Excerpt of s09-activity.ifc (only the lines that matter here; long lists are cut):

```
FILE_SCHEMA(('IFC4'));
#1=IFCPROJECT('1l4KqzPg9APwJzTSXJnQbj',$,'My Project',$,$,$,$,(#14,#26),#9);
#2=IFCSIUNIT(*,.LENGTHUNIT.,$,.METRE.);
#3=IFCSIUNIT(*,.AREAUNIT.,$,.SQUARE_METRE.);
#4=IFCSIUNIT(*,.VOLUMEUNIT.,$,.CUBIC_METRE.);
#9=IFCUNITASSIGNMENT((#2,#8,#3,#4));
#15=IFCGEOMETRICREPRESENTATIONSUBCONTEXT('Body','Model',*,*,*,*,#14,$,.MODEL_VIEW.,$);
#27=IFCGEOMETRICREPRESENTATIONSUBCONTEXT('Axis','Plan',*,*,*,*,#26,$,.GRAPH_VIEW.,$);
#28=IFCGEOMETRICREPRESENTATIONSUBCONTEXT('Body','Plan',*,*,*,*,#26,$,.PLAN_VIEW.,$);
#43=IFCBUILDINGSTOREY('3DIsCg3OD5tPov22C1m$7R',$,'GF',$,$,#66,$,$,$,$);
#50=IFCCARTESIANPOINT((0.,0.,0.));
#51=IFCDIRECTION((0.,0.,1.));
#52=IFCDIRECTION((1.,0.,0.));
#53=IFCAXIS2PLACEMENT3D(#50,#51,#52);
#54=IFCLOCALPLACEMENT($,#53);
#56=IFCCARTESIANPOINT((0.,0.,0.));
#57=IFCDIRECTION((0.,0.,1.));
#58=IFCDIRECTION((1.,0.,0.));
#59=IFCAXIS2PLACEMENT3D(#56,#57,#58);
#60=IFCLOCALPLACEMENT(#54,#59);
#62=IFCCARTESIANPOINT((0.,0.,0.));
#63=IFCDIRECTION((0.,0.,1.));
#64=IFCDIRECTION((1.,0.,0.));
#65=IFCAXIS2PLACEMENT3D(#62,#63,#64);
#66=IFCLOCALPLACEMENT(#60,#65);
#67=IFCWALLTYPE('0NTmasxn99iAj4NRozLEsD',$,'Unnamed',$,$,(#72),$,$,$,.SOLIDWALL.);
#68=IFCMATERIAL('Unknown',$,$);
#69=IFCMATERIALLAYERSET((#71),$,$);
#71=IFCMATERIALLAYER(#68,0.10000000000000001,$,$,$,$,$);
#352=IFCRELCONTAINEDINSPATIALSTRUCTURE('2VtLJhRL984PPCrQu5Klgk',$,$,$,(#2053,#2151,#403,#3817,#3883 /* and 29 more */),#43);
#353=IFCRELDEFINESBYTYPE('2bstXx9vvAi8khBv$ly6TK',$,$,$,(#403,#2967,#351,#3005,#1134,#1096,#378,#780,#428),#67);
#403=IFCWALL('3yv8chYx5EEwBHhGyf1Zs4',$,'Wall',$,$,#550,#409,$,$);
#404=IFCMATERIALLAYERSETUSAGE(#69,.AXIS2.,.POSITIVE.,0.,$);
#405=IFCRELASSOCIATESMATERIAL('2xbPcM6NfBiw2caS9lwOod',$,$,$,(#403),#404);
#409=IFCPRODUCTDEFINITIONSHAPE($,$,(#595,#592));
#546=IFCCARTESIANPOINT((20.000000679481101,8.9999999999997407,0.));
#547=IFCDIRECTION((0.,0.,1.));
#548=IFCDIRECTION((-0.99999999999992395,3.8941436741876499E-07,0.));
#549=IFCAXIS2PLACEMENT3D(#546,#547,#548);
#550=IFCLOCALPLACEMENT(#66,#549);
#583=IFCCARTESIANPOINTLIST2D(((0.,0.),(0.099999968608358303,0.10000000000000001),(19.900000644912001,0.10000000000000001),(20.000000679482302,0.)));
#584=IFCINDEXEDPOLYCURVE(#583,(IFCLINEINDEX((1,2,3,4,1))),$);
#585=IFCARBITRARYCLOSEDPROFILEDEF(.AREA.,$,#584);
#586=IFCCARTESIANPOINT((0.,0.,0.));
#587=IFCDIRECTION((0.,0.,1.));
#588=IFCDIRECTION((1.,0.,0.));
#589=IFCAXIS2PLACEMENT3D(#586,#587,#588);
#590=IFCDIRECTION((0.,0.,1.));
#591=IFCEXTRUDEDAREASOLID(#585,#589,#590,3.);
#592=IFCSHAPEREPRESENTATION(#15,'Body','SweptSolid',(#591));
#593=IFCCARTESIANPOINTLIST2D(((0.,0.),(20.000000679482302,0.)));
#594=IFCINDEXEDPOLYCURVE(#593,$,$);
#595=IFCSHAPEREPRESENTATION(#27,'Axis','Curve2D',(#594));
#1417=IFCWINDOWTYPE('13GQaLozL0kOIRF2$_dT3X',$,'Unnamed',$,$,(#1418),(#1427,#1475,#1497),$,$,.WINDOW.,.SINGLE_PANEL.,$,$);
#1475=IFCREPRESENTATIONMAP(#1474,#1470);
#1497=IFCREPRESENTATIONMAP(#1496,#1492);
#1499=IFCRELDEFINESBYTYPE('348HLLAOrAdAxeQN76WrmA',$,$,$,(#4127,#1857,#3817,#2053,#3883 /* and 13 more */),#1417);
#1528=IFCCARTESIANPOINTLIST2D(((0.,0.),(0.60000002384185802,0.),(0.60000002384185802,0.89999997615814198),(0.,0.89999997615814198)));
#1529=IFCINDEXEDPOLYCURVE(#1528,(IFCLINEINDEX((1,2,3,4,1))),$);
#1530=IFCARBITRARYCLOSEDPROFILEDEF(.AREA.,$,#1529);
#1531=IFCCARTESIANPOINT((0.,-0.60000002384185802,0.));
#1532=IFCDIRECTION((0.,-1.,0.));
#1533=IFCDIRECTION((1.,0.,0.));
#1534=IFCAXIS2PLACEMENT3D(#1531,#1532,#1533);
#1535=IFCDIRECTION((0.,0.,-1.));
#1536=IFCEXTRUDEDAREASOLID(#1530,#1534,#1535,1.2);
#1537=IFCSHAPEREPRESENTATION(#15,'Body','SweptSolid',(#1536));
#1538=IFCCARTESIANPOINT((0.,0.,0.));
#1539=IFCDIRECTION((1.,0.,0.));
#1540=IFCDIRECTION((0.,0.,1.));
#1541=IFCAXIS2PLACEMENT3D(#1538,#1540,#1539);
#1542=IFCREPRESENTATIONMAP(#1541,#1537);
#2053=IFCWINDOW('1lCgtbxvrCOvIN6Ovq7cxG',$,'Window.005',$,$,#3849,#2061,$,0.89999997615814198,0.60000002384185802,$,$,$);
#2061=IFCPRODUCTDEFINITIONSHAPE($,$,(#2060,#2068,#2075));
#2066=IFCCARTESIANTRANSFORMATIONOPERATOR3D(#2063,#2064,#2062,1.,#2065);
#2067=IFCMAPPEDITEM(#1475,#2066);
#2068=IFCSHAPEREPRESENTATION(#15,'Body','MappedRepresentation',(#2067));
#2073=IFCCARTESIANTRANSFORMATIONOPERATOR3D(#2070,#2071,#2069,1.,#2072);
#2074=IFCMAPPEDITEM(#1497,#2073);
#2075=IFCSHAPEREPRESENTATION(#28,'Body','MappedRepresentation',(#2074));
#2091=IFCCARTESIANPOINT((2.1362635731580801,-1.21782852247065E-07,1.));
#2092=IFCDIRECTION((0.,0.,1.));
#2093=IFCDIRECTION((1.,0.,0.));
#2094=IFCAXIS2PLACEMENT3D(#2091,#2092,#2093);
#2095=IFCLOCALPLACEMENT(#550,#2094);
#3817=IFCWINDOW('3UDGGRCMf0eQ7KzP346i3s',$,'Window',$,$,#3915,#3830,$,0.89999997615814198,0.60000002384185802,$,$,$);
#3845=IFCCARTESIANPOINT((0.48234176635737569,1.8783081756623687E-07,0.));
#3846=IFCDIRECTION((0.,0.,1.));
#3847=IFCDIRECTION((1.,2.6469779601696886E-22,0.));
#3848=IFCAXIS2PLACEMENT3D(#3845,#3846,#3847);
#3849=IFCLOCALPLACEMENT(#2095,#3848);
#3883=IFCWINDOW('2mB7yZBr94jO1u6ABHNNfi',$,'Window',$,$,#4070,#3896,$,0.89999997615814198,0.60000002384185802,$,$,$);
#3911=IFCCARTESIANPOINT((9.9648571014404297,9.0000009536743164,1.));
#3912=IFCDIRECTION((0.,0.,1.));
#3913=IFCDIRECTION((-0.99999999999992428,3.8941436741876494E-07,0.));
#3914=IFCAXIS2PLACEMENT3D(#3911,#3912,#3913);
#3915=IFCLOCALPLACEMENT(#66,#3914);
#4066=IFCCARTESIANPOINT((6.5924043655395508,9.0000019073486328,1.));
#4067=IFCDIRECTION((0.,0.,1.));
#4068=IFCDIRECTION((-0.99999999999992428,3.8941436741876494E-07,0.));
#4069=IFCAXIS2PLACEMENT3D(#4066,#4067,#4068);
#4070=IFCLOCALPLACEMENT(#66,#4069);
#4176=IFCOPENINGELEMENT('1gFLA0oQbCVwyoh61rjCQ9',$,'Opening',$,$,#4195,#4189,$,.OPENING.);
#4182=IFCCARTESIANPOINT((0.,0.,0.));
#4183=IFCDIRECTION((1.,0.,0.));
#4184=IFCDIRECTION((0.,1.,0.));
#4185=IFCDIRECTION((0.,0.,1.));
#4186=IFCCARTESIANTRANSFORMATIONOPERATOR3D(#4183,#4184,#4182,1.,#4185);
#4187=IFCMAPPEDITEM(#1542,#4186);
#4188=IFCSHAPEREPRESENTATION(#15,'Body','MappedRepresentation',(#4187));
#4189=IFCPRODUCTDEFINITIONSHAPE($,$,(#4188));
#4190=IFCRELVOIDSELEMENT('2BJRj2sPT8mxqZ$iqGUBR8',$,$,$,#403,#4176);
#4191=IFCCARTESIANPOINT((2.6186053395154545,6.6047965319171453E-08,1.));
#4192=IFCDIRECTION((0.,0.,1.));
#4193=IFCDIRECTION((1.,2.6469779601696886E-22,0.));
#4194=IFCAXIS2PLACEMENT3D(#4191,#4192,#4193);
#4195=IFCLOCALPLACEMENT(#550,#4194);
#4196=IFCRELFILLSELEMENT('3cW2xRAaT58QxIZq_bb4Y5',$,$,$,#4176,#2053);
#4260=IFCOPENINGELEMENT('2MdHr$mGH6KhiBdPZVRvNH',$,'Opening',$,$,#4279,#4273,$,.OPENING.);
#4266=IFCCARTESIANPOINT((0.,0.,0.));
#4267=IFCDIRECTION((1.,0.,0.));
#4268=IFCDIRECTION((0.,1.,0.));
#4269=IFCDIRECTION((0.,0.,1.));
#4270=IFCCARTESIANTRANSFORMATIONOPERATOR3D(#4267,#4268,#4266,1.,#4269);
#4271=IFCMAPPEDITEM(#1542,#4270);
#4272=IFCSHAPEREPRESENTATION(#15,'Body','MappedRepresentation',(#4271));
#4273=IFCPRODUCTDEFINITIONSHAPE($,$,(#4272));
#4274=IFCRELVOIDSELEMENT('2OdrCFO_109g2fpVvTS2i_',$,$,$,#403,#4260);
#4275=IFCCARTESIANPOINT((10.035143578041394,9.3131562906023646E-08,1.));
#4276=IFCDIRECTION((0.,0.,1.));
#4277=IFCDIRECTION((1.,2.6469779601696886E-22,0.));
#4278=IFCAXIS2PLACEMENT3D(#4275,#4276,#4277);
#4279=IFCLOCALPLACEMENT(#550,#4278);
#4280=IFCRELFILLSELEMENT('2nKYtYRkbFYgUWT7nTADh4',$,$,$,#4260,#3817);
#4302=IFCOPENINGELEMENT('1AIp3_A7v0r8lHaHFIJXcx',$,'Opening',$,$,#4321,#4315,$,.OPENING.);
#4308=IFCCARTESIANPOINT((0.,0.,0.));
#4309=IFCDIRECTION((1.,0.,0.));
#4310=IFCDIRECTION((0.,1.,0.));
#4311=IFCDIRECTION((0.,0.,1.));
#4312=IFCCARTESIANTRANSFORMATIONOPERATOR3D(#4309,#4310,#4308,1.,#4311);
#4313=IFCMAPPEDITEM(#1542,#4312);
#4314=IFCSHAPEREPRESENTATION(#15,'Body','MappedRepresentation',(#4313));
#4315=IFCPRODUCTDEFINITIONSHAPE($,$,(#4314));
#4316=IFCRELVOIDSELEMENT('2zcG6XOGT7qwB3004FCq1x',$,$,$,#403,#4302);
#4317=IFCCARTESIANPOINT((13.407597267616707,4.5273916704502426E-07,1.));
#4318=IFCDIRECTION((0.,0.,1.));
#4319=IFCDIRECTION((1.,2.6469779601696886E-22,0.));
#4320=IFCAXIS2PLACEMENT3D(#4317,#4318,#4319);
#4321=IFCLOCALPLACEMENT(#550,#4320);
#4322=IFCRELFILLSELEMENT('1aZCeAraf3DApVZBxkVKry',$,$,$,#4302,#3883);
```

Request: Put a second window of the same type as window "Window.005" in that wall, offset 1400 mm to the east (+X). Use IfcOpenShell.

```python
import ifcopenshell
import ifcopenshell.api.feature
import ifcopenshell.api.geometry
import ifcopenshell.api.root
import ifcopenshell.geom
import ifcopenshell.util.element
import ifcopenshell.util.placement
import ifcopenshell.util.shape
import ifcopenshell.util.unit

model = ifcopenshell.open("s09-activity.ifc")
unit_scale = ifcopenshell.util.unit.calculate_unit_scale(model)
settings = ifcopenshell.geom.settings()


def volume(element):
    """Net volume in cubic metres, openings subtracted."""
    shape = ifcopenshell.geom.create_shape(settings, element)
    return ifcopenshell.util.shape.get_volume(shape.geometry)


window = model.by_guid("1lCgtbxvrCOvIN6Ovq7cxG")
opening = window.FillsVoids[0].RelatingOpeningElement
wall = opening.VoidsElements[0].RelatingBuildingElement
before = volume(wall)
shift = ifcopenshell.util.placement.get_local_placement(wall.ObjectPlacement)[:3, 0] * -1.4 / unit_scale

# copy_class copies the void relationship, type, container and properties, but no geometry.
new_opening = ifcopenshell.api.root.copy_class(model, product=opening)
new_opening.Representation = ifcopenshell.util.element.copy_deep(
    model, opening.Representation, exclude=["IfcGeometricRepresentationContext", "IfcRepresentationMap"]
)
new_window = ifcopenshell.api.root.copy_class(model, product=window)
new_window.Representation = ifcopenshell.util.element.copy_deep(
    model, window.Representation, exclude=["IfcGeometricRepresentationContext", "IfcRepresentationMap"]
)
ifcopenshell.api.feature.add_filling(model, opening=new_opening, element=new_window)

for old, new in ((opening, new_opening), (window, new_window)):
    matrix = ifcopenshell.util.placement.get_local_placement(old.ObjectPlacement)
    matrix[:3, 3] += shift
    ifcopenshell.api.geometry.edit_object_placement(model, product=new, matrix=matrix, is_si=False)

after = volume(wall)

print(f"wall volume {before:.3f} -> {after:.3f} m3")

model.write("s09-activity_edited.ifc")
```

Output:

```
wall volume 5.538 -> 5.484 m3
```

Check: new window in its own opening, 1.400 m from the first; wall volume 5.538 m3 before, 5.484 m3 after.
